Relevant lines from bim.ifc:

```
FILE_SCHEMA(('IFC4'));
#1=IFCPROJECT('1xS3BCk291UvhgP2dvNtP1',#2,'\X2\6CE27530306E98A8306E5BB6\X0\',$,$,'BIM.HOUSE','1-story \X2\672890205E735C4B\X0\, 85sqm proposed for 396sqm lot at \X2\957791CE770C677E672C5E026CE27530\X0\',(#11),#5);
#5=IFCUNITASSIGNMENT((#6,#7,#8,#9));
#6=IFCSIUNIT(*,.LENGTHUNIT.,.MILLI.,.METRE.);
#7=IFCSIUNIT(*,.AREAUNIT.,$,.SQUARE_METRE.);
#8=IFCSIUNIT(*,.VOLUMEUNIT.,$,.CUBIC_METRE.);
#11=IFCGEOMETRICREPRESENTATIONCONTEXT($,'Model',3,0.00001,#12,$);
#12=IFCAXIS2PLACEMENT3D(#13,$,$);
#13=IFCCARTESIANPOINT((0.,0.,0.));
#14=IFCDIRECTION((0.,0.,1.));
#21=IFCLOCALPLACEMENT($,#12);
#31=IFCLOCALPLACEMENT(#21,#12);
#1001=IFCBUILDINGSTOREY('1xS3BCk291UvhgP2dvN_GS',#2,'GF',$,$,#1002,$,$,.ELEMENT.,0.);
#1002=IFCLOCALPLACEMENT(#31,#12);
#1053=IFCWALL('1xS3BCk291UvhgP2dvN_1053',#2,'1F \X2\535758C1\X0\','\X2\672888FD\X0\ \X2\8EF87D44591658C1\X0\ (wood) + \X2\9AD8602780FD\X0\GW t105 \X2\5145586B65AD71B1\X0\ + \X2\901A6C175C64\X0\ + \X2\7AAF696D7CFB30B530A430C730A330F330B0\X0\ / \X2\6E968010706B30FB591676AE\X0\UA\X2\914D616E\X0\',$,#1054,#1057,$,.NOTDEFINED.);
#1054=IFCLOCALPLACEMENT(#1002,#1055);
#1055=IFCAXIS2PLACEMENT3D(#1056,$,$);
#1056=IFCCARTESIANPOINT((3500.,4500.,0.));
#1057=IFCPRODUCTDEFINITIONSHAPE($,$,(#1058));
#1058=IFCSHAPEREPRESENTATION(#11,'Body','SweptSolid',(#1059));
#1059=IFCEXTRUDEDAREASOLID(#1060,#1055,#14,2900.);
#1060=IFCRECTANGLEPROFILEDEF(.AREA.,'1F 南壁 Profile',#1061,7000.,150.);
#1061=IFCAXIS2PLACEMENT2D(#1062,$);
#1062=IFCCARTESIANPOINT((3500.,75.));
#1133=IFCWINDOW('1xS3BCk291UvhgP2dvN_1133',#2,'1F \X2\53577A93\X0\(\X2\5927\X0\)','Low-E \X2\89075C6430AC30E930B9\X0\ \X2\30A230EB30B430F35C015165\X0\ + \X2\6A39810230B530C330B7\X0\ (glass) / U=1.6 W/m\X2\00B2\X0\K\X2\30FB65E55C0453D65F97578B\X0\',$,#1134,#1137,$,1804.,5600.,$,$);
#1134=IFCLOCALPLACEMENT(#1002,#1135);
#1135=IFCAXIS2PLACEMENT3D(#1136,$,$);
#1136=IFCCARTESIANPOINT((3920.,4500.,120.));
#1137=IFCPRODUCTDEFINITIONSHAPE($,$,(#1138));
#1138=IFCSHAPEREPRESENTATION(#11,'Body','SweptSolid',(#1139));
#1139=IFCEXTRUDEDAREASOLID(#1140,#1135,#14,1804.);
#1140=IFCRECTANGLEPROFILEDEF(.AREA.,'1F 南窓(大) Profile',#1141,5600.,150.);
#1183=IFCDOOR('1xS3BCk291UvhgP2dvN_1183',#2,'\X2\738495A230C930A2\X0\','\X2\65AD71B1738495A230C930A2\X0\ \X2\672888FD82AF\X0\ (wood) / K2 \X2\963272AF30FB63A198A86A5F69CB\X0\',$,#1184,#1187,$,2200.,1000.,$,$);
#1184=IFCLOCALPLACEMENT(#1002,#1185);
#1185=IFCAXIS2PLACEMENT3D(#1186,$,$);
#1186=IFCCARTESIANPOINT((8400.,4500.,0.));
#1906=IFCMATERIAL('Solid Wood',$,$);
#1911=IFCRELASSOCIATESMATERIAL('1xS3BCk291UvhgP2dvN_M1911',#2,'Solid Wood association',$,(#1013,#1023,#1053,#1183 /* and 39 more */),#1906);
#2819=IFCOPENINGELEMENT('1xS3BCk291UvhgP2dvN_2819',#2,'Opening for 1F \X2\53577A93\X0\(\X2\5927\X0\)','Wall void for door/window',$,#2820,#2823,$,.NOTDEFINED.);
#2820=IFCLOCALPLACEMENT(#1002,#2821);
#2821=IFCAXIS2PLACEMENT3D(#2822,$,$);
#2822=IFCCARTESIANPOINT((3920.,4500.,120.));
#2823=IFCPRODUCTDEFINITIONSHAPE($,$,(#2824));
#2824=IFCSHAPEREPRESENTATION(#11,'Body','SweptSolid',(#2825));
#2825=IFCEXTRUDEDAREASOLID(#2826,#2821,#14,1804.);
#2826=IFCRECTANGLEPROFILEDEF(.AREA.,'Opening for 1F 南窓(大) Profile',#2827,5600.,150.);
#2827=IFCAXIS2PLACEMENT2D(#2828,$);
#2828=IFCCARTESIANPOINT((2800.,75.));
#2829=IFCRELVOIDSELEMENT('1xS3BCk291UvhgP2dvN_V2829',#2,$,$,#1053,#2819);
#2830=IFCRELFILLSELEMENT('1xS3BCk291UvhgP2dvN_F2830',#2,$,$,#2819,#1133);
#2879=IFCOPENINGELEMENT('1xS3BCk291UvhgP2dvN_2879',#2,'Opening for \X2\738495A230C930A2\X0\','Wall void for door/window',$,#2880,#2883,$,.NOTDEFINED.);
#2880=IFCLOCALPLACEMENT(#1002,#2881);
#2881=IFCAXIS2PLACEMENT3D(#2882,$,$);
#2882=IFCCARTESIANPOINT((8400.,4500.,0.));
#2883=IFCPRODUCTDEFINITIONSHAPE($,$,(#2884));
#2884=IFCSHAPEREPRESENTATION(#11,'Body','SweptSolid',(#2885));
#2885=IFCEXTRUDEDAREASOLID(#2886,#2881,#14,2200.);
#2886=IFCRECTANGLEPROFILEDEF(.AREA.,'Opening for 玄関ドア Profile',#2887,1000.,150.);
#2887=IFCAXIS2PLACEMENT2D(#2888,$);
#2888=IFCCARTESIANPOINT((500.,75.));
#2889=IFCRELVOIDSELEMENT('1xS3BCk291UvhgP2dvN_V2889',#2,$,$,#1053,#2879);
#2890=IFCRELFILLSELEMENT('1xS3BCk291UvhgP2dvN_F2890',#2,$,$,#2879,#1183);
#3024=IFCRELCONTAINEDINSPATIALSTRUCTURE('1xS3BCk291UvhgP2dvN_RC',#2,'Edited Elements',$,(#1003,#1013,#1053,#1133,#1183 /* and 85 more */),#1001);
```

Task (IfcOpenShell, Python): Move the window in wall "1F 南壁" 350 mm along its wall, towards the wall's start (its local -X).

```python
import ifcopenshell
import ifcopenshell.api.geometry
import ifcopenshell.util.placement
import ifcopenshell.util.unit

model = ifcopenshell.open("bim.ifc")
unit_scale = ifcopenshell.util.unit.calculate_unit_scale(model)

window = model.by_guid("1xS3BCk291UvhgP2dvN_1133")
opening = window.FillsVoids[0].RelatingOpeningElement
wall = opening.VoidsElements[0].RelatingBuildingElement

wall_matrix = ifcopenshell.util.placement.get_local_placement(wall.ObjectPlacement)
shift = wall_matrix[:3, 0] * -0.35 / unit_scale
before = ifcopenshell.util.placement.get_local_placement(window.ObjectPlacement)[:3, 3].copy()

# The window is not placed relative to its opening, so move both.
for product in (opening, window):
    matrix = ifcopenshell.util.placement.get_local_placement(product.ObjectPlacement)
    matrix[:3, 3] += shift
    ifcopenshell.api.geometry.edit_object_placement(model, product=product, matrix=matrix, is_si=False)

after = ifcopenshell.util.placement.get_local_placement(window.ObjectPlacement)[:3, 3]
print("window moved by", (after - before).round(3) + 0.0)

model.write("bim-out.ifc")
```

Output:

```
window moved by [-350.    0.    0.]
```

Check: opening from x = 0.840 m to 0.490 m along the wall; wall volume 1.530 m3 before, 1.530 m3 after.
